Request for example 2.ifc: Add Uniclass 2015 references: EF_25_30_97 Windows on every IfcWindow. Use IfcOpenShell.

First a look at what the model holds.

```python
import ifcopenshell

model = ifcopenshell.open("example 2.ifc")
print(model.schema)
print("classifications:", [c.Name for c in model.by_type("IfcClassification")])
for ifc_class in ("IfcDoor", "IfcRoof", "IfcStair", "IfcWall", "IfcWindow"):
    print(ifc_class, len(model.by_type(ifc_class)))
```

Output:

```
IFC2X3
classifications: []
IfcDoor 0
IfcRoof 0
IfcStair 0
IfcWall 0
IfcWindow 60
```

```python
import ifcopenshell
import ifcopenshell.api.classification

model = ifcopenshell.open("example 2.ifc")

# IFC2X3 requires Source and Edition and has no link from the project to the system.
system = model.create_entity("IfcClassification", Source="NBS", Edition="2015", Name="Uniclass 2015")

codes = {
    "IfcWindow": ("EF_25_30_97", "Windows"),
}
for ifc_class, (code, name) in codes.items():
    products = model.by_type(ifc_class)
    ifcopenshell.api.classification.add_reference(
        model, products=products, classification=system, identification=code, name=name
    )
    print(code, len(products))

model.write("example 2-out.ifc")
```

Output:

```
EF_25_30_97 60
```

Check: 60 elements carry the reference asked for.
